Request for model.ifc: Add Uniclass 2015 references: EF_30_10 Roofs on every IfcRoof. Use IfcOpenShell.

First a look at what the model holds.

```python
import ifcopenshell

model = ifcopenshell.open("model.ifc")
print(model.schema)
print("classifications:", [c.Name for c in model.by_type("IfcClassification")])
for ifc_class in ("IfcDoor", "IfcRoof", "IfcStair", "IfcWall", "IfcWindow"):
    print(ifc_class, len(model.by_type(ifc_class)))
```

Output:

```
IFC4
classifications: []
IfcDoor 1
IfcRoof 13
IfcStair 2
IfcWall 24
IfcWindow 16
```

```python
import ifcopenshell
import ifcopenshell.api.classification

model = ifcopenshell.open("model.ifc")

system = ifcopenshell.api.classification.add_classification(model, classification="Uniclass 2015")

codes = {
    "IfcRoof": ("EF_30_10", "Roofs"),
}
for ifc_class, (code, name) in codes.items():
    products = model.by_type(ifc_class)
    ifcopenshell.api.classification.add_reference(
        model, products=products, classification=system, identification=code, name=name
    )
    print(code, len(products))

model.write("model_updated.ifc")
```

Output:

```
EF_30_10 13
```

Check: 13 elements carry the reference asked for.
